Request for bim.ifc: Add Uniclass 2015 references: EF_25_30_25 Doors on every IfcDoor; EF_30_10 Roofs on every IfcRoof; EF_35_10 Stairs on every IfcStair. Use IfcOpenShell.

First a look at what the model holds.

```python
import ifcopenshell

model = ifcopenshell.open("bim.ifc")
print(model.schema)
print("classifications:", [c.Name for c in model.by_type("IfcClassification")])
for ifc_class in ("IfcDoor", "IfcRoof", "IfcStair", "IfcWall", "IfcWindow"):
    print(ifc_class, len(model.by_type(ifc_class)))
```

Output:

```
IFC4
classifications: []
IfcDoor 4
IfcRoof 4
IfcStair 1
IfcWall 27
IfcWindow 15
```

```python
import ifcopenshell
import ifcopenshell.api.classification

model = ifcopenshell.open("bim.ifc")

system = ifcopenshell.api.classification.add_classification(model, classification="Uniclass 2015")

codes = {
    "IfcDoor": ("EF_25_30_25", "Doors"),
    "IfcRoof": ("EF_30_10", "Roofs"),
    "IfcStair": ("EF_35_10", "Stairs"),
}
for ifc_class, (code, name) in codes.items():
    products = model.by_type(ifc_class)
    ifcopenshell.api.classification.add_reference(
        model, products=products, classification=system, identification=code, name=name
    )
    print(code, len(products))

model.write("bim_v2.ifc")
```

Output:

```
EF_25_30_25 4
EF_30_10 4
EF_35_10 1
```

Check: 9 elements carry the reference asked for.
